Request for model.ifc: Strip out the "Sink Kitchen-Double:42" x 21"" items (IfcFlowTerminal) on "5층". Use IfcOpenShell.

First a look at what the model holds.

```python
import ifcopenshell
import ifcopenshell.util.element

model = ifcopenshell.open("model.ifc")
print(model.schema)
storey = next(s for s in model.by_type("IfcBuildingStorey") if s.Name == "5층")
terminals = [e for e in ifcopenshell.util.element.get_decomposition(storey) if e.is_a("IfcFlowTerminal")]
seen = {}
for e in terminals:
    element_type = ifcopenshell.util.element.get_type(e)
    name = element_type.Name if element_type not in (None, e) else None
    seen[name] = seen.get(name, 0) + 1
for name, count in sorted(seen.items(), key=str):
    print(count, "x", name)
```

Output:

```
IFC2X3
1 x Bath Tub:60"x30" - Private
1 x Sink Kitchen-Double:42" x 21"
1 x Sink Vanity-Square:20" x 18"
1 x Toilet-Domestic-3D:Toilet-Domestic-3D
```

```python
import ifcopenshell
import ifcopenshell.api.root
import ifcopenshell.util.element

model = ifcopenshell.open("model.ifc")

storey = next(s for s in model.by_type("IfcBuildingStorey") if s.Name == "5층")
terminals = [e for e in ifcopenshell.util.element.get_decomposition(storey) if e.is_a("IfcFlowTerminal")]
targets = [e for e in terminals if (t := ifcopenshell.util.element.get_type(e)) not in (None, e) and t.Name == 'Sink Kitchen-Double:42" x 21"']

for e in targets:
    ifcopenshell.api.root.remove_product(model, product=e)
print(len(targets), "removed")

model.write("model_rev.ifc")
```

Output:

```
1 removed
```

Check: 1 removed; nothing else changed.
